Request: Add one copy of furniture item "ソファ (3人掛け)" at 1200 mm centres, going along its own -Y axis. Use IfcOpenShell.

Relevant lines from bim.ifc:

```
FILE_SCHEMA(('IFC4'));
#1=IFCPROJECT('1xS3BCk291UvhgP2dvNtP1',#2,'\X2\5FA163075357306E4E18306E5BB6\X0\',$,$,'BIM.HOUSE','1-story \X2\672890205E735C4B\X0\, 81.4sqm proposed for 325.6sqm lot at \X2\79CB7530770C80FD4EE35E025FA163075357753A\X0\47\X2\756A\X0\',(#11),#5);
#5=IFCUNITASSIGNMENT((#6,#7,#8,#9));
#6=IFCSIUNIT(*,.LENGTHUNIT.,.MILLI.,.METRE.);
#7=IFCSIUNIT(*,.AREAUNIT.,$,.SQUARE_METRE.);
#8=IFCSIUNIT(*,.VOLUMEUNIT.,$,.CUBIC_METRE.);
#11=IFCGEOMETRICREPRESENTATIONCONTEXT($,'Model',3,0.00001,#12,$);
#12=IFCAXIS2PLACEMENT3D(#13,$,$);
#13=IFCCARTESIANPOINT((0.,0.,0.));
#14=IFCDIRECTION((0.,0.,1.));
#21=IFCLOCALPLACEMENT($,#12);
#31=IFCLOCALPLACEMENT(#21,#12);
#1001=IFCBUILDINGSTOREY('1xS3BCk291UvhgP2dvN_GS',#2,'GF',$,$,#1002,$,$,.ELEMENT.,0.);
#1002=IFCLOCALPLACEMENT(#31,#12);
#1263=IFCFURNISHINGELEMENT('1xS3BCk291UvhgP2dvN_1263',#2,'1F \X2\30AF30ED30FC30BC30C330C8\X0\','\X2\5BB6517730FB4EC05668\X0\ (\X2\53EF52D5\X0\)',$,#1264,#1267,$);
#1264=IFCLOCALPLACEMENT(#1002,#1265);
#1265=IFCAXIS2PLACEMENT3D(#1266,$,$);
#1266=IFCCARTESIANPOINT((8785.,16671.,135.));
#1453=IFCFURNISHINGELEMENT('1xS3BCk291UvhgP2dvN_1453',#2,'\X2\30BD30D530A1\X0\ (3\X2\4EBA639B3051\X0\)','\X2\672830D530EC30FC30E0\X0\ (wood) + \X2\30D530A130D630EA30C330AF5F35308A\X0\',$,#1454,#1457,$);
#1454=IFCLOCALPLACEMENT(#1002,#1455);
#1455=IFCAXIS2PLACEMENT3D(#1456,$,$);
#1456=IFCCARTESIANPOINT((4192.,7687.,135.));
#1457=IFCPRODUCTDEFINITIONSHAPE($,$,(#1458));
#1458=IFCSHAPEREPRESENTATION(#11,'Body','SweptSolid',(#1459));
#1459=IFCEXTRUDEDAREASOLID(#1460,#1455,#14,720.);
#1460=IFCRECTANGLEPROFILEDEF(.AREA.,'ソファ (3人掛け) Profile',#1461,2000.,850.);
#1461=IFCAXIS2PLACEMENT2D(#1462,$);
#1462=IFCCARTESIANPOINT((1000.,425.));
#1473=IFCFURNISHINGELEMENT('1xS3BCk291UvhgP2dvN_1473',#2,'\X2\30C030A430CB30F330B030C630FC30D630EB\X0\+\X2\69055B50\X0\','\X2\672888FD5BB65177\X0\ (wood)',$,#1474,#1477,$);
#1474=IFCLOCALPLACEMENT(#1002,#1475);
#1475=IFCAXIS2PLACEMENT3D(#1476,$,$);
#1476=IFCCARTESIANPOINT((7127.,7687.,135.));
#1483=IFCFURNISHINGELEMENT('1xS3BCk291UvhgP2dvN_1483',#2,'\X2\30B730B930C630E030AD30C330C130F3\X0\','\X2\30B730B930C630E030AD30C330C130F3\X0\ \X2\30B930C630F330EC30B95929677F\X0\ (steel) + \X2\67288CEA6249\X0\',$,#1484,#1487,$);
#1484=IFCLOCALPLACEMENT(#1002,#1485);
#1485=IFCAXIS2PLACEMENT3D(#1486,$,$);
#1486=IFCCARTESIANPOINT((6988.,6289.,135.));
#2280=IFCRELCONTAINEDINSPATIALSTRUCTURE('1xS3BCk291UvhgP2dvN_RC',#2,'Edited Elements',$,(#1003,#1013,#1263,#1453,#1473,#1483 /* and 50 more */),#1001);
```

```python
import ifcopenshell
import ifcopenshell.api.geometry
import ifcopenshell.api.root
import ifcopenshell.util.element
import ifcopenshell.util.placement
import ifcopenshell.util.unit

model = ifcopenshell.open("bim.ifc")
unit_scale = ifcopenshell.util.unit.calculate_unit_scale(model)


def reuse_history(source, copy):
    """copy_class also copies each property set's owner history, people and application; keep the originals."""
    for rel in copy.IsDefinedBy:
        if rel.is_a("IfcRelDefinesByProperties") and (history := rel.RelatingPropertyDefinition.OwnerHistory):
            rel.RelatingPropertyDefinition.OwnerHistory = source.OwnerHistory
            ifcopenshell.util.element.remove_deep2(model, history)


source = model.by_id(1453)
base = ifcopenshell.util.placement.get_local_placement(source.ObjectPlacement)
step = -base[:3, 1] * 1.2 / unit_scale

for i in range(1, 2):
    copy = ifcopenshell.api.root.copy_class(model, product=source)
    copy.Representation = ifcopenshell.util.element.copy_deep(
        model, source.Representation, exclude=["IfcGeometricRepresentationContext", "IfcRepresentationMap"]
    )
    reuse_history(source, copy)
    matrix = base.copy()
    matrix[:3, 3] += i * step
    print("added at", matrix[:3, 3].round(3) + 0.0)
    ifcopenshell.api.geometry.edit_object_placement(model, product=copy, matrix=matrix, is_si=False)

model.write("bim_updated.ifc")
```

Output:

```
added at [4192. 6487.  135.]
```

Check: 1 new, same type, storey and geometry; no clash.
